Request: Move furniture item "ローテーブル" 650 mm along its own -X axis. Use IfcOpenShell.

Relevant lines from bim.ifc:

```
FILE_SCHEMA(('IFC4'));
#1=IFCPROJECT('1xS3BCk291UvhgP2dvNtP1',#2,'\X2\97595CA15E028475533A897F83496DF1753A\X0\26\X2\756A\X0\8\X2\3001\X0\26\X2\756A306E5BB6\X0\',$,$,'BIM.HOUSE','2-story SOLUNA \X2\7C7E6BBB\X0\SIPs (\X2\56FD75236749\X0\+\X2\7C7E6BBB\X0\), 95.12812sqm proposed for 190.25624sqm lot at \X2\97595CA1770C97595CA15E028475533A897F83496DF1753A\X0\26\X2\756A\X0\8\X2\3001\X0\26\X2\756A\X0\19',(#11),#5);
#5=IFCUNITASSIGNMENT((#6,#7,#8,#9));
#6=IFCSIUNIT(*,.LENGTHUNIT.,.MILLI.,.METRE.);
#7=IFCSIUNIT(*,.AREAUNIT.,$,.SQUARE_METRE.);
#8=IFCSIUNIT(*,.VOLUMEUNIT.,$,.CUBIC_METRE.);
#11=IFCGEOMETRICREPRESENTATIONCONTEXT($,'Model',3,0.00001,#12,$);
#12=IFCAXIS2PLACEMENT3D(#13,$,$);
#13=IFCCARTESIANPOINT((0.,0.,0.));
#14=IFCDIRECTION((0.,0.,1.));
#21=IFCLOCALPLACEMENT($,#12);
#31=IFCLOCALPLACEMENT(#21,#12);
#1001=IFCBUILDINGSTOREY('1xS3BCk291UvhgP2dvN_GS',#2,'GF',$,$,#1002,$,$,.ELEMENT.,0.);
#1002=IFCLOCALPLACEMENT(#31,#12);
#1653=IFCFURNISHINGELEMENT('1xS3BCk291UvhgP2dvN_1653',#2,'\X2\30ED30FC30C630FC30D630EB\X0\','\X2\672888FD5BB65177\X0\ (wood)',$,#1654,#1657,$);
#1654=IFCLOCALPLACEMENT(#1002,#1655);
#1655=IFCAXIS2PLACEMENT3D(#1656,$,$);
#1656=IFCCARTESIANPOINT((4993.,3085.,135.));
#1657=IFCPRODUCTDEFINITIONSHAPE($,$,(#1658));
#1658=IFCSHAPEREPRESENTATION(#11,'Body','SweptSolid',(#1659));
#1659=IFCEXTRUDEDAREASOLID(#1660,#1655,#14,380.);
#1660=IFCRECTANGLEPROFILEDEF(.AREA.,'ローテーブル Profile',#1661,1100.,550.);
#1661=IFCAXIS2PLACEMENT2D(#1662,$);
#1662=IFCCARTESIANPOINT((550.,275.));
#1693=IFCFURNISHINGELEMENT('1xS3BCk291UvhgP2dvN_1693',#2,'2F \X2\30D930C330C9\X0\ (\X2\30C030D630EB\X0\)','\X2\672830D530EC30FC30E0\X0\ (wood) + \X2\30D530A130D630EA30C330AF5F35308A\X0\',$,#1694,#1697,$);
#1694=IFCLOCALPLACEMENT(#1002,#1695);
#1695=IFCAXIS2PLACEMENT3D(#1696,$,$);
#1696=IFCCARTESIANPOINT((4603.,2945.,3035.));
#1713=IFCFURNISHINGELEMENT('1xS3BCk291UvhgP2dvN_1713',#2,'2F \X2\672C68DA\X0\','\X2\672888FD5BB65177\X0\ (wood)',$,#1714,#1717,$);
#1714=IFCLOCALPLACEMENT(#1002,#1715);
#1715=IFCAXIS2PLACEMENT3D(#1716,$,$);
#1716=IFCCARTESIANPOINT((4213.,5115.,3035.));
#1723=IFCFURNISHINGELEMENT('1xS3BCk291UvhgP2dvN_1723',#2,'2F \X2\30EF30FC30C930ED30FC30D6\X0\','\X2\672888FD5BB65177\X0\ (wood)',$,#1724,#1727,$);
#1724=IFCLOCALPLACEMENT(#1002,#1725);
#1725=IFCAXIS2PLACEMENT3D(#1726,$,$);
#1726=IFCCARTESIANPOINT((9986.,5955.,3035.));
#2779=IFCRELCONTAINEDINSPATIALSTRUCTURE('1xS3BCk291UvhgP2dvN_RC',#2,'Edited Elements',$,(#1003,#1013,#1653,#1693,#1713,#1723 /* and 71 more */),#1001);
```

```python
import ifcopenshell
import ifcopenshell.api.geometry
import ifcopenshell.util.placement

model = ifcopenshell.open("bim.ifc")

item = model.by_guid("1xS3BCk291UvhgP2dvN_1653")
matrix = ifcopenshell.util.placement.get_local_placement(item.ObjectPlacement)
matrix[:3, 3] -= matrix[:3, 0] * 650.0
ifcopenshell.api.geometry.edit_object_placement(model, product=item, matrix=matrix, is_si=False)

print(ifcopenshell.util.placement.get_local_placement(item.ObjectPlacement).round(3) + 0.0)

model.write("bim-out.ifc")
```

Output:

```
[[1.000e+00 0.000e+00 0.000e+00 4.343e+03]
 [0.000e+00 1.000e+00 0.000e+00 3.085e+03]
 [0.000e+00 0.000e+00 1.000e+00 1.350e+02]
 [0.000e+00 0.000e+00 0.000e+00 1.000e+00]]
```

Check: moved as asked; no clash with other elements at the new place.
